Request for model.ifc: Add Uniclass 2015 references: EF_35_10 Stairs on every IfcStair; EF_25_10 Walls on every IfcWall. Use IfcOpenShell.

First a look at what the model holds.

```python
import ifcopenshell

model = ifcopenshell.open("model.ifc")
print(model.schema)
print("classifications:", [c.Name for c in model.by_type("IfcClassification")])
for ifc_class in ("IfcDoor", "IfcRoof", "IfcStair", "IfcWall", "IfcWindow"):
    print(ifc_class, len(model.by_type(ifc_class)))
```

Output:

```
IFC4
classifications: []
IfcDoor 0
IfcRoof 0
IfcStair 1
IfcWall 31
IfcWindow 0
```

```python
import ifcopenshell
import ifcopenshell.api.classification

model = ifcopenshell.open("model.ifc")

system = ifcopenshell.api.classification.add_classification(model, classification="Uniclass 2015")

codes = {
    "IfcStair": ("EF_35_10", "Stairs"),
    "IfcWall": ("EF_25_10", "Walls"),
}
for ifc_class, (code, name) in codes.items():
    products = model.by_type(ifc_class)
    ifcopenshell.api.classification.add_reference(
        model, products=products, classification=system, identification=code, name=name
    )
    print(code, len(products))

model.write("model_v2.ifc")
```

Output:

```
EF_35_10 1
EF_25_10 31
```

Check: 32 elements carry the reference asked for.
